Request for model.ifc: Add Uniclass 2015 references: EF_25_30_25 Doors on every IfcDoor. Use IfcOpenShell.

First a look at what the model holds.

```python
import ifcopenshell

model = ifcopenshell.open("model.ifc")
print(model.schema)
print("classifications:", [c.Name for c in model.by_type("IfcClassification")])
for ifc_class in ("IfcDoor", "IfcRoof", "IfcStair", "IfcWall", "IfcWindow"):
    print(ifc_class, len(model.by_type(ifc_class)))
```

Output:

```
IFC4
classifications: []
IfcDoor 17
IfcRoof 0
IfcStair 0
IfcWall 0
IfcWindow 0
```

```python
import ifcopenshell
import ifcopenshell.api.classification

model = ifcopenshell.open("model.ifc")

system = ifcopenshell.api.classification.add_classification(model, classification="Uniclass 2015")

codes = {
    "IfcDoor": ("EF_25_30_25", "Doors"),
}
for ifc_class, (code, name) in codes.items():
    products = model.by_type(ifc_class)
    ifcopenshell.api.classification.add_reference(
        model, products=products, classification=system, identification=code, name=name
    )
    print(code, len(products))

model.write("model_v2.ifc")
```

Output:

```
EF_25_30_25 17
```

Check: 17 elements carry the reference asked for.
